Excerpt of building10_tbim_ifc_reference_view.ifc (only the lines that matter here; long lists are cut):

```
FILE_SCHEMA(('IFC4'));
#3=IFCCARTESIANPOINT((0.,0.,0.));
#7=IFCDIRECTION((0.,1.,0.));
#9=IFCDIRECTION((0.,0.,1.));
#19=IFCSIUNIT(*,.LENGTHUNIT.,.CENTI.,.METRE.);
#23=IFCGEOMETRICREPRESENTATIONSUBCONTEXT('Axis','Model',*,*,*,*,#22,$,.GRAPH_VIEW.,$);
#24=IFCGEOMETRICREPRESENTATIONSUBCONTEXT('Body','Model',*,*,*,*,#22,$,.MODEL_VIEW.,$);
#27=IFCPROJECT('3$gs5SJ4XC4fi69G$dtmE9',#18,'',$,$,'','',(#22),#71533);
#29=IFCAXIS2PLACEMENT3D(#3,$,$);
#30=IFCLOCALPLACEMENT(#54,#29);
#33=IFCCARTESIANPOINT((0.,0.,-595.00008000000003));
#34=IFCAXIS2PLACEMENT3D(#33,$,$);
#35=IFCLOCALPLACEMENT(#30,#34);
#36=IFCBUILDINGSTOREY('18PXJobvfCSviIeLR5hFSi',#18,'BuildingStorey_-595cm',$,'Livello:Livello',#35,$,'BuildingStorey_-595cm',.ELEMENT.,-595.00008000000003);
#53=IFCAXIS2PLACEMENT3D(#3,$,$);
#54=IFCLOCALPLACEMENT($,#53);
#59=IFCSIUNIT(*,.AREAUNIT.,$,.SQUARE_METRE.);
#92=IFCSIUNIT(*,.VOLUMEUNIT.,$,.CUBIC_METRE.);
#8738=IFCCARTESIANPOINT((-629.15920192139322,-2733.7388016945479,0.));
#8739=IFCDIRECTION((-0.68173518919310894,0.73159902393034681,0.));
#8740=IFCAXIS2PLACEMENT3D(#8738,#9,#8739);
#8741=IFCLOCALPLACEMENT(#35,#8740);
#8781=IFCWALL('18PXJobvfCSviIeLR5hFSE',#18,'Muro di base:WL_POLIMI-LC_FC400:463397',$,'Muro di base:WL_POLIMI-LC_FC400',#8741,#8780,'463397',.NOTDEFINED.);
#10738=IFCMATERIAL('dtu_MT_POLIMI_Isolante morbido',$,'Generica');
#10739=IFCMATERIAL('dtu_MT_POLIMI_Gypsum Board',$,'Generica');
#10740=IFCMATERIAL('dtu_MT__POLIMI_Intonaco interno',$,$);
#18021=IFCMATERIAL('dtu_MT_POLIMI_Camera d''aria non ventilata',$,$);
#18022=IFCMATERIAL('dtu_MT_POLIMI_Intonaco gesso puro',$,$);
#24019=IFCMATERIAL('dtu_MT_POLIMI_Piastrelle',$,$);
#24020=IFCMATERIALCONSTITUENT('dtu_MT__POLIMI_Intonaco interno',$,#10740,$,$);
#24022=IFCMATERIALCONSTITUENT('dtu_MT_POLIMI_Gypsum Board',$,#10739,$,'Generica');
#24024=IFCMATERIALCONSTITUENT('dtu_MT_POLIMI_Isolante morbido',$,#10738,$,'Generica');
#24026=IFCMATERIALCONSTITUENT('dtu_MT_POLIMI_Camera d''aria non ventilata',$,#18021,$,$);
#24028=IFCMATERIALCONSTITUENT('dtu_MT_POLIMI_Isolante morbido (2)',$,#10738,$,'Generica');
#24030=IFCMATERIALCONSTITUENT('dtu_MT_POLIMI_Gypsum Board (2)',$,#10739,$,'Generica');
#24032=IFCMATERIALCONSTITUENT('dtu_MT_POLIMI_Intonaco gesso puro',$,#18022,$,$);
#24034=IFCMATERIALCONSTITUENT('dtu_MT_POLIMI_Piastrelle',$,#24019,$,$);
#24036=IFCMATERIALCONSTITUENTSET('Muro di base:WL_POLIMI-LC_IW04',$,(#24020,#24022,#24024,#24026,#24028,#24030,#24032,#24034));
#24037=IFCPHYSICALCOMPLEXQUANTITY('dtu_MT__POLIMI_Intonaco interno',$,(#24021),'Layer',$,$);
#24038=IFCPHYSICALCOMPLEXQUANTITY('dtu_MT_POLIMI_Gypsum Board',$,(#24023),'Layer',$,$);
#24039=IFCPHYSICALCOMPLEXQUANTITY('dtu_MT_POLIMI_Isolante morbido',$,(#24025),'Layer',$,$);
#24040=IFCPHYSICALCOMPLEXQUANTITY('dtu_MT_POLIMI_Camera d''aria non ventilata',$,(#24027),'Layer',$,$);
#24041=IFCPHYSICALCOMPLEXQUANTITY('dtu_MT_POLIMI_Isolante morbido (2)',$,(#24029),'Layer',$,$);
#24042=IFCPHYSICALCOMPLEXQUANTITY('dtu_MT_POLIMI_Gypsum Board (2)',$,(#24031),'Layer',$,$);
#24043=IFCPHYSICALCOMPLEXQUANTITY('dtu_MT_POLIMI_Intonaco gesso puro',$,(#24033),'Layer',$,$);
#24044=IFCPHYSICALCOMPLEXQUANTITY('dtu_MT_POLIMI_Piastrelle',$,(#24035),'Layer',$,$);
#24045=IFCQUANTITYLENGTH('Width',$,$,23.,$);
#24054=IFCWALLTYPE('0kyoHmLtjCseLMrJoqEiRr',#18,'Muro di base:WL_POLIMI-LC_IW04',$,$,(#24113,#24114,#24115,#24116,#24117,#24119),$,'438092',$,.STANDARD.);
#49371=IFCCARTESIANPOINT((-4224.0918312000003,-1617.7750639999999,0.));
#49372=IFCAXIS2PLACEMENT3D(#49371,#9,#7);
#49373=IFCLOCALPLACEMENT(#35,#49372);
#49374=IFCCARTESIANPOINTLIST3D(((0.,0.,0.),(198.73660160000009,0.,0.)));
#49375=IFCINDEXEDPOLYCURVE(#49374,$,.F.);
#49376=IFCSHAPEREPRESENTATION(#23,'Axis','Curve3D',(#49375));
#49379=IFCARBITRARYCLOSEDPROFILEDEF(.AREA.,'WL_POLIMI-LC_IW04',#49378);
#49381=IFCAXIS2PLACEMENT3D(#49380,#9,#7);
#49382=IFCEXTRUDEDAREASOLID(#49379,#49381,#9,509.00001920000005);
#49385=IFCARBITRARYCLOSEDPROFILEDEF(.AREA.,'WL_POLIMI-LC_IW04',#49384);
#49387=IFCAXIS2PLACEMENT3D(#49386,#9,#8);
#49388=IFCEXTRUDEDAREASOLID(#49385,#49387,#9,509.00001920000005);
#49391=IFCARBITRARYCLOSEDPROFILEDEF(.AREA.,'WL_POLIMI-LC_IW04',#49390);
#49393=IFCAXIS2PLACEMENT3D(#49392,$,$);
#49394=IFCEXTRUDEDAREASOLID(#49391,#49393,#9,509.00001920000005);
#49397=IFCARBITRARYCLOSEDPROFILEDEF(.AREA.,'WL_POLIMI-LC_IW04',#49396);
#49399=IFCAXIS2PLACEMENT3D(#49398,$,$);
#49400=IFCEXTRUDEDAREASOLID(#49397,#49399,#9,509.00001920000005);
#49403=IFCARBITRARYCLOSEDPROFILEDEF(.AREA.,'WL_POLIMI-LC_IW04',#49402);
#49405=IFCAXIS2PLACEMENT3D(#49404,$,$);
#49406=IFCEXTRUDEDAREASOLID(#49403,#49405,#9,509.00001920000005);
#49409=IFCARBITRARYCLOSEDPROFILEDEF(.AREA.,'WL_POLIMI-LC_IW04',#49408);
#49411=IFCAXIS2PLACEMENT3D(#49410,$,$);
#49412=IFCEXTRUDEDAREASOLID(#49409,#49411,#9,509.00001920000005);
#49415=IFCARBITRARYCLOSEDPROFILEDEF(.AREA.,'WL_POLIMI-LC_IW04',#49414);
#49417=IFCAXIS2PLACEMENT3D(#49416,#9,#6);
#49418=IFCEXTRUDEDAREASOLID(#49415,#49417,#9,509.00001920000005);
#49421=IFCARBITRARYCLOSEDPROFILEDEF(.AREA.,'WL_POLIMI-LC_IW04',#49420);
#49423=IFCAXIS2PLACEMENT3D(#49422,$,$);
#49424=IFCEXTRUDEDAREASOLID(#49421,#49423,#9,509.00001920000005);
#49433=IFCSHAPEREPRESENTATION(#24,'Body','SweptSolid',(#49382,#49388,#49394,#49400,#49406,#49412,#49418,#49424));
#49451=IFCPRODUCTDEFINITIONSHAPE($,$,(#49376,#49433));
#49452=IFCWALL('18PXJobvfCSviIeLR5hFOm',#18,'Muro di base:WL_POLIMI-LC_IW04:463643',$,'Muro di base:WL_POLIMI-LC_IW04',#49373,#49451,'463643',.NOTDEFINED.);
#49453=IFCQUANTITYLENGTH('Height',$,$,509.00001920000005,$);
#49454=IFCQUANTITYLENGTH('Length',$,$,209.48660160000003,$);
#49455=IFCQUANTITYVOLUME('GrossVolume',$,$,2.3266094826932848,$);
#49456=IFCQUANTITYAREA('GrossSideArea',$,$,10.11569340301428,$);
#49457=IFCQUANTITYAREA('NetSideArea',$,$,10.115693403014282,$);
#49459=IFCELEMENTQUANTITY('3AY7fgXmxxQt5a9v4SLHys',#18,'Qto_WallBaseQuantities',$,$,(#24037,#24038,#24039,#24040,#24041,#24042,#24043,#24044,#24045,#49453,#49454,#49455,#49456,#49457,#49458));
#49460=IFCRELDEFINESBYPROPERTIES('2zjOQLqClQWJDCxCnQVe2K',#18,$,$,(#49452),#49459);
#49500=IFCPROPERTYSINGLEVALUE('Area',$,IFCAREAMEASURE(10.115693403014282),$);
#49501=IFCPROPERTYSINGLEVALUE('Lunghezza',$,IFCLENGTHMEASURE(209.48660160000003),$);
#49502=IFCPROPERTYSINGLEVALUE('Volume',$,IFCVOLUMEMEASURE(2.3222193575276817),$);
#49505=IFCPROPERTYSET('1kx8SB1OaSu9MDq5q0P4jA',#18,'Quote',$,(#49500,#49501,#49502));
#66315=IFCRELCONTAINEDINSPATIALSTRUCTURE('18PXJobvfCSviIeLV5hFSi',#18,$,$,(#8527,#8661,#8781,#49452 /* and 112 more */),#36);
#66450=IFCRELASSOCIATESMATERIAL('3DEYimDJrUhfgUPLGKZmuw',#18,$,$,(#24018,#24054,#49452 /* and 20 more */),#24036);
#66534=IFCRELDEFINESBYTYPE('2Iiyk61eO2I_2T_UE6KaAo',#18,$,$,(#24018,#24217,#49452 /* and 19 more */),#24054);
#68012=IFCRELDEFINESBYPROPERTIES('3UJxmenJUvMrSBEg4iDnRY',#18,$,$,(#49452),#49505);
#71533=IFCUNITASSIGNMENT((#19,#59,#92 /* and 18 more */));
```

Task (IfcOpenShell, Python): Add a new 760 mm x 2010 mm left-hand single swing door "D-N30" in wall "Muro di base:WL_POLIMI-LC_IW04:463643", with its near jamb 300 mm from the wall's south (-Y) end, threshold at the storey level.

```python
import numpy as np
import ifcopenshell
import ifcopenshell.api.feature
import ifcopenshell.api.geometry
import ifcopenshell.api.pset
import ifcopenshell.api.root
import ifcopenshell.api.spatial
import ifcopenshell.geom
import ifcopenshell.util.element
import ifcopenshell.util.placement
import ifcopenshell.util.representation
import ifcopenshell.util.shape
import ifcopenshell.util.unit

model = ifcopenshell.open("building10_tbim_ifc_reference_view.ifc")
unit_scale = ifcopenshell.util.unit.calculate_unit_scale(model)
area_scale = ifcopenshell.util.unit.calculate_unit_scale(model, "AREAUNIT")
volume_scale = ifcopenshell.util.unit.calculate_unit_scale(model, "VOLUMEUNIT")
settings = ifcopenshell.geom.settings()


def volume(element):
    """Net volume in cubic metres, openings subtracted."""
    shape = ifcopenshell.geom.create_shape(settings, element)
    return ifcopenshell.util.shape.get_volume(shape.geometry)


wall = model.by_id(49452)
storey = ifcopenshell.util.element.get_container(wall, ifc_class="IfcBuildingStorey")
context = ifcopenshell.util.representation.get_context(model, "Model", "Body", "MODEL_VIEW")
before = volume(wall)

width, height, from_end, sill = 0.76, 2.01, 0.3, 0.0  # metres

# The wall runs along its own X axis, and the end named is its -X end.
wall_shape = ifcopenshell.geom.create_shape(settings, wall)
x, y, z = ifcopenshell.util.shape.get_vertices(wall_shape.geometry).T
start = x.min() + from_end
face, thickness = float(y.min()), float(y.max() - y.min())
wall_matrix = ifcopenshell.util.placement.get_local_placement(wall.ObjectPlacement)
level = ifcopenshell.util.placement.get_local_placement(storey.ObjectPlacement)[2, 3]


def in_wall(x, y):
    """Placement at x, y metres in the wall's axes, at sill height."""
    matrix = wall_matrix.copy()
    matrix[:, 3] = wall_matrix @ np.array([x / unit_scale, y / unit_scale, 0.0, 1.0])
    matrix[2, 3] = level + sill / unit_scale
    return matrix


# Opening: a box that overshoots both wall faces by 50 mm.
opening = ifcopenshell.api.root.create_entity(model, ifc_class="IfcOpeningElement", predefined_type="OPENING")
box = ifcopenshell.api.geometry.add_wall_representation(
    model, context=context, length=width, height=height, thickness=thickness + 0.1
)
ifcopenshell.api.geometry.assign_representation(model, product=opening, representation=box)
ifcopenshell.api.geometry.edit_object_placement(model, product=opening, matrix=in_wall(start, face - 0.05), is_si=False)
ifcopenshell.api.feature.add_feature(model, feature=opening, element=wall)

door = ifcopenshell.api.root.create_entity(model, ifc_class="IfcDoor", name="D-N30", predefined_type="DOOR")
door.OverallWidth, door.OverallHeight = width / unit_scale, height / unit_scale
door.OperationType = "SINGLE_SWING_LEFT"
body = ifcopenshell.api.geometry.add_door_representation(
    model,
    context=context,
    overall_width=door.OverallWidth,
    overall_height=door.OverallHeight,
    operation_type="SINGLE_SWING_LEFT",
    lining_properties={"LiningDepth": thickness / unit_scale, "ThresholdDepth": thickness / unit_scale},
)
ifcopenshell.api.geometry.assign_representation(model, product=door, representation=body)
ifcopenshell.api.spatial.assign_container(model, products=[door], relating_structure=storey)
ifcopenshell.api.feature.add_filling(model, opening=opening, element=door)

# The lining spans the wall, so the door starts at the wall face.
ifcopenshell.api.geometry.edit_object_placement(model, product=door, matrix=in_wall(start, face), is_si=False)

after = volume(wall)

# Update the wall's stored quantities.
qto = model.by_id(ifcopenshell.util.element.get_pset(wall, "Qto_WallBaseQuantities", should_inherit=False)["id"])
ifcopenshell.api.pset.edit_qto(model, qto=qto, properties={
    "NetSideArea": after / thickness / area_scale,
    "NetVolume": after / volume_scale,
})
pset = model.by_id(ifcopenshell.util.element.get_pset(wall, "Quote", should_inherit=False)["id"])
ifcopenshell.api.pset.edit_pset(model, pset=pset, properties={
    "Area": model.create_entity("IfcAreaMeasure", after / thickness / area_scale),
    "Volume": model.create_entity("IfcVolumeMeasure", after / volume_scale),
})

print(f"wall volume {before:.3f} -> {after:.3f} m3")

model.write("building10_tbim_ifc_reference_view_updated.ifc")
```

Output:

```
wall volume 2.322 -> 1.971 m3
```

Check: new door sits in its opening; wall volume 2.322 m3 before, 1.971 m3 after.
